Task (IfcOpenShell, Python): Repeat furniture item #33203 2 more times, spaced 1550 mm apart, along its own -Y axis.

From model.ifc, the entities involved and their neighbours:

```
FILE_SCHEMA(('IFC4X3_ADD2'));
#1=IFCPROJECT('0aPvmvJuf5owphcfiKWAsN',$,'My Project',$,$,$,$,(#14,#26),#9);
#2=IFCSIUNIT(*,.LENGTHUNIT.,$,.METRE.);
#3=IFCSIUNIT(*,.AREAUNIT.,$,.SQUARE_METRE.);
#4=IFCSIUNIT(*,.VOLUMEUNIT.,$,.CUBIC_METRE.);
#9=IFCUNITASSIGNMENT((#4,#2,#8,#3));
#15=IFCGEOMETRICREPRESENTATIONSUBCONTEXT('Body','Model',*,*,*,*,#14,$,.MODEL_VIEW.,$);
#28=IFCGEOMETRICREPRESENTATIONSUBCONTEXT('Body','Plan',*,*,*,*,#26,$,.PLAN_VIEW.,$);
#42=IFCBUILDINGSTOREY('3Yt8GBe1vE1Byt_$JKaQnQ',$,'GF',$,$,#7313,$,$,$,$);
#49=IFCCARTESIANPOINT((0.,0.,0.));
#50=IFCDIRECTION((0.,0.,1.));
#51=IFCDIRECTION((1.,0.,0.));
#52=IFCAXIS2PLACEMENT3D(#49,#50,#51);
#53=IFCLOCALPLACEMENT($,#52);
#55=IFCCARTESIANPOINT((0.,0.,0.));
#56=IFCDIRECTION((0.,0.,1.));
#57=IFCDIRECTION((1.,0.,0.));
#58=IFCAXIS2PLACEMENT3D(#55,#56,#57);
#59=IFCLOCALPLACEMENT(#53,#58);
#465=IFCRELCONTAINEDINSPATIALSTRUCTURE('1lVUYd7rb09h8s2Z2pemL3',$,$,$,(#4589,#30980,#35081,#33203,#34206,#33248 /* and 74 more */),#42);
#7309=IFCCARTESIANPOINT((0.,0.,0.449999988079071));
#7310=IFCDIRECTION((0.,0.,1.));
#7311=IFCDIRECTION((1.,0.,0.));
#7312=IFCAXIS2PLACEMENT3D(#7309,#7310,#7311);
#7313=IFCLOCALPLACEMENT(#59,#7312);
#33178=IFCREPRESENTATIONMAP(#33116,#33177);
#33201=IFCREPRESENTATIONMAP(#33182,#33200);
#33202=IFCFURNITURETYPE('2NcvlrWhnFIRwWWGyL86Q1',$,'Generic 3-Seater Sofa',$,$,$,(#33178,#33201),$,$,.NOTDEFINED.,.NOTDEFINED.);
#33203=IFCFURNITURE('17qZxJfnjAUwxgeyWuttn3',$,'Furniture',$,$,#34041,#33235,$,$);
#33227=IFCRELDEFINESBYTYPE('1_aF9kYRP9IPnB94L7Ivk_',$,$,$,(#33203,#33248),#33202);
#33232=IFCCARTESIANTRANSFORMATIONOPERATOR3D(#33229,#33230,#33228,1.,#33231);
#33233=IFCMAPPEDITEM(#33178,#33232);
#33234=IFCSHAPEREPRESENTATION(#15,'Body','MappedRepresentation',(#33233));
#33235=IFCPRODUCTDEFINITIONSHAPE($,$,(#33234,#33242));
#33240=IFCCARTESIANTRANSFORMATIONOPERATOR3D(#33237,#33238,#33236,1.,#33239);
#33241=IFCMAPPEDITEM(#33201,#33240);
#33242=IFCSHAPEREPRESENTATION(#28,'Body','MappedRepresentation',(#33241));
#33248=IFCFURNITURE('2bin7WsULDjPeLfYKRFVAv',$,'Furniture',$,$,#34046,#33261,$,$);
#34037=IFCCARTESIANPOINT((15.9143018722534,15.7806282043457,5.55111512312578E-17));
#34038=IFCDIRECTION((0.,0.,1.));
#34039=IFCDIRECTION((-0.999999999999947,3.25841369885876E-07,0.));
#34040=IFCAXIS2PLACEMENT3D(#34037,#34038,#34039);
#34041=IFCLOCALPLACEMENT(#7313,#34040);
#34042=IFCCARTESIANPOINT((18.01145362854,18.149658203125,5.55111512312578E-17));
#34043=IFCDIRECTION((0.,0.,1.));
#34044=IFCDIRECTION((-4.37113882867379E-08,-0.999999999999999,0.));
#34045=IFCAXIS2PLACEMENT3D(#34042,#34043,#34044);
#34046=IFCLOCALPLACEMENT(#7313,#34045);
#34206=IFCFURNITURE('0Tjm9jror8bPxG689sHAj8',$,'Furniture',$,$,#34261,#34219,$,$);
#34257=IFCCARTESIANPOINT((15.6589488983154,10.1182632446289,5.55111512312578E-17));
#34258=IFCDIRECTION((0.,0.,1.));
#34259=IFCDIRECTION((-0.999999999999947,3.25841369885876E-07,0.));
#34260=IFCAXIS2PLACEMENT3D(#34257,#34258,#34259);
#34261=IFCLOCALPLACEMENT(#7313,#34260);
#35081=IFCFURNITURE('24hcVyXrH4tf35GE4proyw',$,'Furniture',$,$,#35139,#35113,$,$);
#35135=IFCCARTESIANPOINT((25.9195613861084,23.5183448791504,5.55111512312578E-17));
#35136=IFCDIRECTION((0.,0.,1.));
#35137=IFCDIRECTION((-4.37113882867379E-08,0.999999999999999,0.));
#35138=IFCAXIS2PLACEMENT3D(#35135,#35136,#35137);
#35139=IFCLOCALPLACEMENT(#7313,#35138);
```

```python
import ifcopenshell
import ifcopenshell.api.geometry
import ifcopenshell.api.root
import ifcopenshell.util.element
import ifcopenshell.util.placement

model = ifcopenshell.open("model.ifc")

source = model.by_guid("17qZxJfnjAUwxgeyWuttn3")
base = ifcopenshell.util.placement.get_local_placement(source.ObjectPlacement)
step = -base[:3, 1] * 1.55

for i in range(1, 3):
    copy = ifcopenshell.api.root.copy_class(model, product=source)
    copy.Representation = ifcopenshell.util.element.copy_deep(
        model, source.Representation, exclude=["IfcGeometricRepresentationContext", "IfcRepresentationMap"]
    )
    matrix = base.copy()
    matrix[:3, 3] += i * step
    print("added at", matrix[:3, 3].round(3) + 0.0)
    ifcopenshell.api.geometry.edit_object_placement(model, product=copy, matrix=matrix, is_si=False)

model.write("model_v2.ifc")
```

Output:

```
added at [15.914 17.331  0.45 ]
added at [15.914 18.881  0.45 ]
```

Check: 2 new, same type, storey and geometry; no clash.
